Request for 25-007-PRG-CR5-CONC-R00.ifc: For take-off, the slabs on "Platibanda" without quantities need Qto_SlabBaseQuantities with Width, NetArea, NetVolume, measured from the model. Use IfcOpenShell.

First a look at what the model holds.

```python
import ifcopenshell
import ifcopenshell.util.element
import ifcopenshell.util.unit

model = ifcopenshell.open("25-007-PRG-CR5-CONC-R00.ifc")
print(model.schema)
for unit_type in ("LENGTHUNIT", "AREAUNIT", "VOLUMEUNIT"):
    print(unit_type, ifcopenshell.util.unit.calculate_unit_scale(model, unit_type))
storey = next(s for s in model.by_type("IfcBuildingStorey") if s.Name == "Platibanda")
slabs = [e for e in ifcopenshell.util.element.get_decomposition(storey) if e.is_a("IfcSlab")]
for e in sorted(slabs, key=lambda e: e.id()):
    print(e.id(), e.is_a(), e.Name, list(ifcopenshell.util.element.get_psets(e, qtos_only=True)), sep=" | ")
```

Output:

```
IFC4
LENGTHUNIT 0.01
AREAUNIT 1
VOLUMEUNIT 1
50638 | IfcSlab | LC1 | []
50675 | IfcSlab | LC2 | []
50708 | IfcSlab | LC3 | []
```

```python
import ifcopenshell
import ifcopenshell.api.pset
import ifcopenshell.geom
import ifcopenshell.util.element
import ifcopenshell.util.shape
import ifcopenshell.util.unit

model = ifcopenshell.open("25-007-PRG-CR5-CONC-R00.ifc")
unit_scale = ifcopenshell.util.unit.calculate_unit_scale(model)
area_scale = ifcopenshell.util.unit.calculate_unit_scale(model, "AREAUNIT")
volume_scale = ifcopenshell.util.unit.calculate_unit_scale(model, "VOLUMEUNIT")
settings = ifcopenshell.geom.settings()

storey = next(s for s in model.by_type("IfcBuildingStorey") if s.Name == "Platibanda")
slabs = [e for e in ifcopenshell.util.element.get_decomposition(storey) if e.is_a("IfcSlab")]

for e in sorted(slabs, key=lambda e: e.id()):
    if ifcopenshell.util.element.get_psets(e, qtos_only=True, should_inherit=False):
        continue
    # Geometry comes back in metres, in the element's own axes.
    shape = ifcopenshell.geom.create_shape(settings, e)
    values = {
        "Width": ifcopenshell.util.shape.get_z(shape.geometry) / unit_scale,
        "NetArea": ifcopenshell.util.shape.get_footprint_area(shape.geometry) / area_scale,
        "NetVolume": ifcopenshell.util.shape.get_volume(shape.geometry) / volume_scale,
    }
    qto = ifcopenshell.api.pset.add_qto(model, product=e, name="Qto_SlabBaseQuantities")
    ifcopenshell.api.pset.edit_qto(model, qto=qto, properties=values)
    print(e.id(), {k: round(v, 3) for k, v in values.items()})

model.write("25-007-PRG-CR5-CONC-R00-out.ifc")
```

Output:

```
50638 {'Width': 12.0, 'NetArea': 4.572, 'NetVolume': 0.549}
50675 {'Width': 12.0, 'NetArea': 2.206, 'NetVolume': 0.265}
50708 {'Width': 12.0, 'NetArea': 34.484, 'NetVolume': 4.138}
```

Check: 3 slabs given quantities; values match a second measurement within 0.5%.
